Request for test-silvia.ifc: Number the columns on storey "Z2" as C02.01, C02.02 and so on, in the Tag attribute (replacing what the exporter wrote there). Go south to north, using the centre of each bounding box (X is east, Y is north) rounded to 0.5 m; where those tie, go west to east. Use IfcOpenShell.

First a look at what the model holds.

```python
import ifcopenshell
import ifcopenshell.util.element
import ifcopenshell.util.placement

model = ifcopenshell.open("test-silvia.ifc")
print(model.schema)
storey = next(s for s in model.by_type("IfcBuildingStorey") if s.Name == "Z2")
columns = [e for e in ifcopenshell.util.element.get_decomposition(storey) if e.is_a("IfcColumn")]
for e in sorted(columns, key=lambda e: e.id()):
    origin = ifcopenshell.util.placement.get_local_placement(e.ObjectPlacement)[:3, 3]
    print(e.id(), e.Tag, e.Name, origin.round(2) + 0.0, sep=" | ")
```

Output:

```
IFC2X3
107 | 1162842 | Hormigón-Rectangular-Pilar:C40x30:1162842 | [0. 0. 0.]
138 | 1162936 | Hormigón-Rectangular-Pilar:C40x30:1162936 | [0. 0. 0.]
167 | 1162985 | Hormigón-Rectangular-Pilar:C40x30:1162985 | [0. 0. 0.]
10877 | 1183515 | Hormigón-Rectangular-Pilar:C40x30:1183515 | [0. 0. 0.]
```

```python
import ifcopenshell
import ifcopenshell.geom
import ifcopenshell.util.element
import ifcopenshell.util.shape

model = ifcopenshell.open("test-silvia.ifc")
settings = ifcopenshell.geom.settings()
settings.set("use-world-coords", True)


def centre(element):
    shape = ifcopenshell.geom.create_shape(settings, element)
    return ifcopenshell.util.shape.get_bbox_centroid(shape.geometry)


storey = next(s for s in model.by_type("IfcBuildingStorey") if s.Name == "Z2")
columns = [e for e in ifcopenshell.util.element.get_decomposition(storey) if e.is_a("IfcColumn")]

# Insertion points can sit at a corner or the storey origin, so sort by the geometry (in metres).
centres = {e: centre(e) for e in columns}
columns.sort(key=lambda e: (round(centres[e][1] / 0.5), centres[e][0]))

for i, e in enumerate(columns, start=1):
    number = f"C02.{i:02d}"
    e.Tag = number
    print(e.id(), number)

model.write("test-silvia_rev.ifc")
```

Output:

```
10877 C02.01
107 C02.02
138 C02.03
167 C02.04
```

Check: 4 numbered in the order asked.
